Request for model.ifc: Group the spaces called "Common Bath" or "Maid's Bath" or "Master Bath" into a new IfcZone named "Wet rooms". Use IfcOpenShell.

First a look at what the model holds.

```python
import ifcopenshell

model = ifcopenshell.open("model.ifc")
print(model.schema)
seen = {}
for space in model.by_type("IfcSpace"):
    seen[space.LongName] = seen.get(space.LongName, 0) + 1
for name, count in sorted(seen.items(), key=str):
    print(count, "x", name)
print("zones:", [z.Name for z in model.by_type("IfcZone")][:20])
```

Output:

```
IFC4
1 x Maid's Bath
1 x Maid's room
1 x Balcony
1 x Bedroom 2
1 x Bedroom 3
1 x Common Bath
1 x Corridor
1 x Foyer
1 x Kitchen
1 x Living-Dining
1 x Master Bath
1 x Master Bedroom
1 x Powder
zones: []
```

```python
import ifcopenshell
import ifcopenshell.api.group
import ifcopenshell.api.root

model = ifcopenshell.open("model.ifc")

names = {"Common Bath", "Maid's Bath", "Master Bath"}
spaces = [s for s in model.by_type("IfcSpace") if s.LongName in names]

zone = ifcopenshell.api.root.create_entity(model, ifc_class="IfcZone", name="Wet rooms")
ifcopenshell.api.group.assign_group(model, products=spaces, group=zone)
print(len(spaces), "spaces in", zone.Name)

model.write("model-out.ifc")
```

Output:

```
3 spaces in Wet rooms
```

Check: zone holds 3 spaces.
